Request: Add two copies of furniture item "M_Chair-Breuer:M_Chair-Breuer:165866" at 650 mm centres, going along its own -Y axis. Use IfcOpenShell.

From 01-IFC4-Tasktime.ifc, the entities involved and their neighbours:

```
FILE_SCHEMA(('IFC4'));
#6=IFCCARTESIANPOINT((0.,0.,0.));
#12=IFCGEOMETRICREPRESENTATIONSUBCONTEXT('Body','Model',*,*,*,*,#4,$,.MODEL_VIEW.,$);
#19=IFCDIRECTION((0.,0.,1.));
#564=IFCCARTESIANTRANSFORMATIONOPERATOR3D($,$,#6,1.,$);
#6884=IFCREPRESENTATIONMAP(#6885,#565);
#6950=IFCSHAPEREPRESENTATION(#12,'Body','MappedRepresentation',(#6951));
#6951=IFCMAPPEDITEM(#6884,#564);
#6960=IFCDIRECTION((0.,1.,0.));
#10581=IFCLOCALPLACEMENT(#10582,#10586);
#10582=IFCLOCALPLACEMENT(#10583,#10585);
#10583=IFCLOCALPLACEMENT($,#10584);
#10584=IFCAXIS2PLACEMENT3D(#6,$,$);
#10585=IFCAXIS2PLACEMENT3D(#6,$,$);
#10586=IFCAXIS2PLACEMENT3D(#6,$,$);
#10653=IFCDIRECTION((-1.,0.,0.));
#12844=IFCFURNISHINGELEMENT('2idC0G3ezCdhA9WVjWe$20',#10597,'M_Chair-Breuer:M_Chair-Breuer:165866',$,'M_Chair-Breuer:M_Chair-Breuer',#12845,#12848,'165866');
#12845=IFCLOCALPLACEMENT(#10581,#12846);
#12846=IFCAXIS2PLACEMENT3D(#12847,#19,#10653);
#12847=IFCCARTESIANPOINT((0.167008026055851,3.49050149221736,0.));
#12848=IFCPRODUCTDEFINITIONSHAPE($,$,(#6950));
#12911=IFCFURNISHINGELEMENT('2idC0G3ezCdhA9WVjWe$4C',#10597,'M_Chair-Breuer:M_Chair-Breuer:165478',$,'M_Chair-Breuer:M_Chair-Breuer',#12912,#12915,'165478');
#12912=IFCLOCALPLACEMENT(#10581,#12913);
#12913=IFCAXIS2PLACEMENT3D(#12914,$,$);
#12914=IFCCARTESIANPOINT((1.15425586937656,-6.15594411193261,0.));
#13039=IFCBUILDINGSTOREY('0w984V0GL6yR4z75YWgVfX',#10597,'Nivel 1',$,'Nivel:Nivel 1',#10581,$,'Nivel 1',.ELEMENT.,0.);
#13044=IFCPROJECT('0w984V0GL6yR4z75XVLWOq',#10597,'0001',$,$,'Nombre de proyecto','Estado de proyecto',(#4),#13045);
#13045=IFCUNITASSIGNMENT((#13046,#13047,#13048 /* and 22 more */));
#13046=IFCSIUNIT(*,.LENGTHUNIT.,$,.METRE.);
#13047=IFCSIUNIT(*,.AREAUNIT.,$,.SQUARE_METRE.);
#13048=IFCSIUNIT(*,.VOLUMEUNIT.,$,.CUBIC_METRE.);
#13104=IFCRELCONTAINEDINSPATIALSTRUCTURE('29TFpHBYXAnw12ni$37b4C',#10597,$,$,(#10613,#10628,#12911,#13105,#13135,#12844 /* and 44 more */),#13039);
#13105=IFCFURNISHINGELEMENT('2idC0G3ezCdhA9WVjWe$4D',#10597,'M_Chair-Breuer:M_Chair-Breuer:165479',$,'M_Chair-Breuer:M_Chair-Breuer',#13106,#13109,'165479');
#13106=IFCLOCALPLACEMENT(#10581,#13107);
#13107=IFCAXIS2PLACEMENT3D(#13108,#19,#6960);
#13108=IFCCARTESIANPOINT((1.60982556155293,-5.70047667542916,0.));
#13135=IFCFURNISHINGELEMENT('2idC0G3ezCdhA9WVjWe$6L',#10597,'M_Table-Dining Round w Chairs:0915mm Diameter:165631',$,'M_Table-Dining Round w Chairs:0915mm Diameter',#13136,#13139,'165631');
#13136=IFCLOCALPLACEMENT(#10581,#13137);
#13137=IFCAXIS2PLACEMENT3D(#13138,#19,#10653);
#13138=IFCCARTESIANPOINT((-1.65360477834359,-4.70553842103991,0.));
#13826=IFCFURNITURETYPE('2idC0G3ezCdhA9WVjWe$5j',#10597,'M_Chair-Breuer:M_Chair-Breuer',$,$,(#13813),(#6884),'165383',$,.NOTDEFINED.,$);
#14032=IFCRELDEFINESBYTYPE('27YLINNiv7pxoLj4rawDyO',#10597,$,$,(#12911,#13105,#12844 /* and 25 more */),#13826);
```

```python
import ifcopenshell
import ifcopenshell.api.geometry
import ifcopenshell.api.root
import ifcopenshell.util.element
import ifcopenshell.util.placement

model = ifcopenshell.open("01-IFC4-Tasktime.ifc")


def reuse_history(source, copy):
    """copy_class also copies each property set's owner history, people and application; keep the originals."""
    for rel in copy.IsDefinedBy:
        if rel.is_a("IfcRelDefinesByProperties") and (history := rel.RelatingPropertyDefinition.OwnerHistory):
            rel.RelatingPropertyDefinition.OwnerHistory = source.OwnerHistory
            ifcopenshell.util.element.remove_deep2(model, history)


source = model.by_guid("2idC0G3ezCdhA9WVjWe$20")
base = ifcopenshell.util.placement.get_local_placement(source.ObjectPlacement)
step = -base[:3, 1] * 0.65

for i in range(1, 3):
    copy = ifcopenshell.api.root.copy_class(model, product=source)
    copy.Representation = ifcopenshell.util.element.copy_deep(
        model, source.Representation, exclude=["IfcGeometricRepresentationContext", "IfcRepresentationMap"]
    )
    copy.Name = "M_Chair-Breuer:M_Chair-Breuer"
    copy.Tag = None
    reuse_history(source, copy)
    matrix = base.copy()
    matrix[:3, 3] += i * step
    print("added at", matrix[:3, 3].round(3) + 0.0)
    ifcopenshell.api.geometry.edit_object_placement(model, product=copy, matrix=matrix, is_si=False)

model.write("01-IFC4-Tasktime_v2.ifc")
```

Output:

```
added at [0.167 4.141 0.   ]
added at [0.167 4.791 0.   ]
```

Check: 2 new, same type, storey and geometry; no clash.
